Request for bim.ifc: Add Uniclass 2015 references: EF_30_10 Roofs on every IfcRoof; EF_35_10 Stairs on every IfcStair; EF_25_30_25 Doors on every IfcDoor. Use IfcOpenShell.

First a look at what the model holds.

```python
import ifcopenshell

model = ifcopenshell.open("bim.ifc")
print(model.schema)
print("classifications:", [c.Name for c in model.by_type("IfcClassification")])
for ifc_class in ("IfcDoor", "IfcRoof", "IfcStair", "IfcWall", "IfcWindow"):
    print(ifc_class, len(model.by_type(ifc_class)))
```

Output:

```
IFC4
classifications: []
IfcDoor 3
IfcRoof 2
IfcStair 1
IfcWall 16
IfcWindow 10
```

```python
import ifcopenshell
import ifcopenshell.api.classification

model = ifcopenshell.open("bim.ifc")

system = ifcopenshell.api.classification.add_classification(model, classification="Uniclass 2015")

codes = {
    "IfcRoof": ("EF_30_10", "Roofs"),
    "IfcStair": ("EF_35_10", "Stairs"),
    "IfcDoor": ("EF_25_30_25", "Doors"),
}
for ifc_class, (code, name) in codes.items():
    products = model.by_type(ifc_class)
    ifcopenshell.api.classification.add_reference(
        model, products=products, classification=system, identification=code, name=name
    )
    print(code, len(products))

model.write("bim_updated.ifc")
```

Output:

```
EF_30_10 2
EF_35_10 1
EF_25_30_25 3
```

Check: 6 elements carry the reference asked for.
